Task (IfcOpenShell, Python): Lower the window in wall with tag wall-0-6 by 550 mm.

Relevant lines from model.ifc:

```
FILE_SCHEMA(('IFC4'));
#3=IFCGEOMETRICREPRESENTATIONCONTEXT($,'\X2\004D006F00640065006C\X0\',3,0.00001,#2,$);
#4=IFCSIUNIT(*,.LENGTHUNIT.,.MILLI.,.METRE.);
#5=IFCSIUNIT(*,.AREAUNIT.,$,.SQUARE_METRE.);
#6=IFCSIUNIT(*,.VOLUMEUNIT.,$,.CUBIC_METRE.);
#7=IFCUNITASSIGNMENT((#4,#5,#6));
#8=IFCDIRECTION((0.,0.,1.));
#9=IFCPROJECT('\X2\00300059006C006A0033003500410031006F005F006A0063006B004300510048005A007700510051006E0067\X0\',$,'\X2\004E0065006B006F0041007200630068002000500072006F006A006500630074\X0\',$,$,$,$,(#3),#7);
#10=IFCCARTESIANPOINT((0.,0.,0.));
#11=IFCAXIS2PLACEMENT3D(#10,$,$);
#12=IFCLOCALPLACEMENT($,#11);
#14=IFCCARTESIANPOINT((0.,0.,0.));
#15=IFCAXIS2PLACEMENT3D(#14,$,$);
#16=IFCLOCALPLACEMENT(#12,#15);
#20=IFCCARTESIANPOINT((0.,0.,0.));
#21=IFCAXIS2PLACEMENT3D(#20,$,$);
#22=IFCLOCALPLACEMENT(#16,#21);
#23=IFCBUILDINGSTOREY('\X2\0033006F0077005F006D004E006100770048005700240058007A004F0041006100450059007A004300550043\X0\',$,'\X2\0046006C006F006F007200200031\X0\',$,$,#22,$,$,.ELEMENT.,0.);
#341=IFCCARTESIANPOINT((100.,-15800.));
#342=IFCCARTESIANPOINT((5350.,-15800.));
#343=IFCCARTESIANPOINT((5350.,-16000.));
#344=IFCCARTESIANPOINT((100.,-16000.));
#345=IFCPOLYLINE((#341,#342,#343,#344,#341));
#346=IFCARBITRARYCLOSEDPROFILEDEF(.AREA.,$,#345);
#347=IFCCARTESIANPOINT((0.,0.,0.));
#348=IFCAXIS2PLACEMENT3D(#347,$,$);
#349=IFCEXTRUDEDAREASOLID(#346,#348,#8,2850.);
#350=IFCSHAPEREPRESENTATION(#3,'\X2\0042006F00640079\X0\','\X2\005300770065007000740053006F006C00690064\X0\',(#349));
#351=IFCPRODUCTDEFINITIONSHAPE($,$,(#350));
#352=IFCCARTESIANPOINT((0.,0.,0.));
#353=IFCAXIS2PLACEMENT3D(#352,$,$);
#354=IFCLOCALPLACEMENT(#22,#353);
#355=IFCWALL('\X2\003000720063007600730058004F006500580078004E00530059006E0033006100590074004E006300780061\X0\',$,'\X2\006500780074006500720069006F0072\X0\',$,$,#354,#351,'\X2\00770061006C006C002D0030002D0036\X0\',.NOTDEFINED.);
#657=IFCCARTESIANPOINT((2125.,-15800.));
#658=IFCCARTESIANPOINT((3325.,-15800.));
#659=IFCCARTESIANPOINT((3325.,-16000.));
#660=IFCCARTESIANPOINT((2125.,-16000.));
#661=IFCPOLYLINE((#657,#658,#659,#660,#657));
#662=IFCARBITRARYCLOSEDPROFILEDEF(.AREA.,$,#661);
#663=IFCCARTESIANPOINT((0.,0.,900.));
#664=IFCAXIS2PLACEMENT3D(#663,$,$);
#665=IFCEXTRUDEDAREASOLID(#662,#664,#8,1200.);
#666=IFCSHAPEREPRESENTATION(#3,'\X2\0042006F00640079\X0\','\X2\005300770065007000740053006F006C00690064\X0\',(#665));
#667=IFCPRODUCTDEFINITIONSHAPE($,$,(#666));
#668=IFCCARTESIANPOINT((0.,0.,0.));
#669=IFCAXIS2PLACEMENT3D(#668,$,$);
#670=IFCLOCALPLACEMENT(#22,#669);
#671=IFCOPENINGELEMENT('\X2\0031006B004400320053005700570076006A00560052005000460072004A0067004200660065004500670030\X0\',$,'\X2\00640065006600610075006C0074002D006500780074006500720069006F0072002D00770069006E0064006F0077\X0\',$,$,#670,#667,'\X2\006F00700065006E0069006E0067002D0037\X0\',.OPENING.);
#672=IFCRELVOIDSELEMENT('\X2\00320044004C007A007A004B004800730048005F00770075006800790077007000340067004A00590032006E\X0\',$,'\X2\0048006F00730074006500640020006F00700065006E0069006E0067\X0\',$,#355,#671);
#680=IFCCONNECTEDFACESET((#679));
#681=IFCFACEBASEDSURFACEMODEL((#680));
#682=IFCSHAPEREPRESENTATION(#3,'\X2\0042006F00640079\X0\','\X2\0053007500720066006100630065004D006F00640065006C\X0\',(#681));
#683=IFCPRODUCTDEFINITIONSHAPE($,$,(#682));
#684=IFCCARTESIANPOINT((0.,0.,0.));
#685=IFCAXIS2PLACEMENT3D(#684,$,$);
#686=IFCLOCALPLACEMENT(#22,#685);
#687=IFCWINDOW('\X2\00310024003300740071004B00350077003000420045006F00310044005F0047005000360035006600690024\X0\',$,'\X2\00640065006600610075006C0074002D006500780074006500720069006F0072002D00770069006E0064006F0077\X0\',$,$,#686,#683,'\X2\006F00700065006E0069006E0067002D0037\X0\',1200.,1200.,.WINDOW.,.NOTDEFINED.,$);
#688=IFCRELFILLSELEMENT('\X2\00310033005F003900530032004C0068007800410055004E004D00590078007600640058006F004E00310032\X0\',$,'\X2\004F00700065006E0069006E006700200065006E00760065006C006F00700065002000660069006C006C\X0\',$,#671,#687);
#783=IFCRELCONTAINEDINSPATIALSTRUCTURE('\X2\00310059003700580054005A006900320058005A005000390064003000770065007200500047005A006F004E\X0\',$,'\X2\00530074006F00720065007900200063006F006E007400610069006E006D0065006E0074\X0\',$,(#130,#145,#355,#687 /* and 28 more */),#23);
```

```python
import numpy as np
import ifcopenshell
import ifcopenshell.api.geometry
import ifcopenshell.util.placement
import ifcopenshell.util.unit

model = ifcopenshell.open("model.ifc")
unit_scale = ifcopenshell.util.unit.calculate_unit_scale(model)

window = model.by_guid("1$3tqK5w0BEo1D_GP65fi$")
opening = window.FillsVoids[0].RelatingOpeningElement
dz = -0.55 / unit_scale

shift = np.array([0.0, 0.0, dz])
# The window is not placed relative to its opening, so move both.
for product in (opening, window):
    matrix = ifcopenshell.util.placement.get_local_placement(product.ObjectPlacement)
    matrix[:3, 3] += shift
    ifcopenshell.api.geometry.edit_object_placement(model, product=product, matrix=matrix, is_si=False)

print(f"moved by {dz * unit_scale:+.3f} m")

model.write("model-out.ifc")
```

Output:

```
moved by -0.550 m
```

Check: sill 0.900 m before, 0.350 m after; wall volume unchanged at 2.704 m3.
